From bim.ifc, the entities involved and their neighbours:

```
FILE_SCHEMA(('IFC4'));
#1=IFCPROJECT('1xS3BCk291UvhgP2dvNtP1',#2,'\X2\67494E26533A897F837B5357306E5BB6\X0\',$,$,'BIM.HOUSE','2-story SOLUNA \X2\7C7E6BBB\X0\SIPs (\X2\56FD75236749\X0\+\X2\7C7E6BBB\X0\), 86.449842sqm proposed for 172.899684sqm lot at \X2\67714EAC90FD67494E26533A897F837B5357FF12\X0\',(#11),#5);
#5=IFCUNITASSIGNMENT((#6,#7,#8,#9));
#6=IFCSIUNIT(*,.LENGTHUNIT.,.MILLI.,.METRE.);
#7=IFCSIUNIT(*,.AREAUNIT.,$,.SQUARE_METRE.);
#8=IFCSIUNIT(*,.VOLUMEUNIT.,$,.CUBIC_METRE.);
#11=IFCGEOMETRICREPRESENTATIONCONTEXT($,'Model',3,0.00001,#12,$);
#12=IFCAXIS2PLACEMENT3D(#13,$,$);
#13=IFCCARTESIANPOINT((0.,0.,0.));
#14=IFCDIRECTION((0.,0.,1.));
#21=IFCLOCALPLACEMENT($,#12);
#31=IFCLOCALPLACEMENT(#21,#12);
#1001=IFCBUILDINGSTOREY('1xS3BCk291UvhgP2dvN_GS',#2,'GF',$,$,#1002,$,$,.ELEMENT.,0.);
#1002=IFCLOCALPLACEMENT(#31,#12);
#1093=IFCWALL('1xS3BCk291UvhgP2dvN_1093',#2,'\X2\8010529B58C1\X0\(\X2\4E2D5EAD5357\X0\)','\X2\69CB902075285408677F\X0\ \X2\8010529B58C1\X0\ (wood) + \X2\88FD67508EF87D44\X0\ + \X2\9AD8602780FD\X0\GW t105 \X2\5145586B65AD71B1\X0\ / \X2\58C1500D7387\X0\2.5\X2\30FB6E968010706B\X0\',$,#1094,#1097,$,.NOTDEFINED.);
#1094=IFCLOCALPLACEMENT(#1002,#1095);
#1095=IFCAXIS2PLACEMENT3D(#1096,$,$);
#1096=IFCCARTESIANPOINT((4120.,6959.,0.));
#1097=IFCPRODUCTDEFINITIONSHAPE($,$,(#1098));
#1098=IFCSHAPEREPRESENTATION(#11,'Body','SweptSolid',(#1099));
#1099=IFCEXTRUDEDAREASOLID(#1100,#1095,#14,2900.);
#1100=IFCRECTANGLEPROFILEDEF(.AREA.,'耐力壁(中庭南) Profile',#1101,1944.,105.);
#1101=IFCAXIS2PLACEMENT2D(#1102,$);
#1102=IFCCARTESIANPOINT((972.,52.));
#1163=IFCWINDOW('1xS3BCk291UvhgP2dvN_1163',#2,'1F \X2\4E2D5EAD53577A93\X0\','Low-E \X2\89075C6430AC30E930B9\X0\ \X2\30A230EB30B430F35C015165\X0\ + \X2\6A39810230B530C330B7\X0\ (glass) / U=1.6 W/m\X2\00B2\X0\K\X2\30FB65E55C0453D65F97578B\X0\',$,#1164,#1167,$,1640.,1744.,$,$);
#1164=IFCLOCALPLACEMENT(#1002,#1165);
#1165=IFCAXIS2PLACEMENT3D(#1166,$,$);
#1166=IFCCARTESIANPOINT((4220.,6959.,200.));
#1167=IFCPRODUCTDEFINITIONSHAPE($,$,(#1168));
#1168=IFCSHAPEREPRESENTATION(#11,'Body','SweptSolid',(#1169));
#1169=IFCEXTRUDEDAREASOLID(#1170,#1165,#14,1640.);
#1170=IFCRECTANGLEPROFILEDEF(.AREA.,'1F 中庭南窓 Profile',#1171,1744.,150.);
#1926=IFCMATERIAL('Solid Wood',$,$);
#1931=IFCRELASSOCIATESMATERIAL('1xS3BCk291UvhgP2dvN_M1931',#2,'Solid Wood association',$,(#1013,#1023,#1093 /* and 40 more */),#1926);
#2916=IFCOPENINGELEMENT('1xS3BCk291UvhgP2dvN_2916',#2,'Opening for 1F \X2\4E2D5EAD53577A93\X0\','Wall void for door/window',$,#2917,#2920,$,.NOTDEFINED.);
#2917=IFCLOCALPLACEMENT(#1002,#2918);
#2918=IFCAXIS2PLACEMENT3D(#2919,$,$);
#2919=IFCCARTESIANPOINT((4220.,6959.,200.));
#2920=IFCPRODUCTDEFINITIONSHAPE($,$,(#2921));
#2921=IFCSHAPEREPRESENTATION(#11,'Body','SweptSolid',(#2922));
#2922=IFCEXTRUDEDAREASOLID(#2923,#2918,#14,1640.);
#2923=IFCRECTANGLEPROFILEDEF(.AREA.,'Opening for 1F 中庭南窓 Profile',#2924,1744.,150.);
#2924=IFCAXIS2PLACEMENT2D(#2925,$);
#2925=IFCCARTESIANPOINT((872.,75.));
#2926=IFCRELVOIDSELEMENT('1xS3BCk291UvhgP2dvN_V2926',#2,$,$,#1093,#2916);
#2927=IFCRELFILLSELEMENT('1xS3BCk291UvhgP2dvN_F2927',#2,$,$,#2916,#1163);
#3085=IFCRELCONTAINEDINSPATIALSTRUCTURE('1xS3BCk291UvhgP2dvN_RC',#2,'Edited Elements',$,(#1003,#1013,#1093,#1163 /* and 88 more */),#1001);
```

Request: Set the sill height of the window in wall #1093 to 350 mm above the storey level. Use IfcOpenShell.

```python
import numpy as np
import ifcopenshell
import ifcopenshell.api.geometry
import ifcopenshell.geom
import ifcopenshell.util.element
import ifcopenshell.util.placement
import ifcopenshell.util.shape
import ifcopenshell.util.unit

model = ifcopenshell.open("bim.ifc")
unit_scale = ifcopenshell.util.unit.calculate_unit_scale(model)

window = model.by_guid("1xS3BCk291UvhgP2dvN_1163")
opening = window.FillsVoids[0].RelatingOpeningElement
storey = ifcopenshell.util.element.get_container(window, ifc_class="IfcBuildingStorey")
level = ifcopenshell.util.placement.get_local_placement(storey.ObjectPlacement)[2, 3]

# The opening's origin need not be at the sill, so measure its lowest point.
shape = ifcopenshell.geom.create_shape(ifcopenshell.geom.settings(), opening)
bottom = ifcopenshell.util.shape.get_shape_bottom_elevation(shape, shape.geometry) / unit_scale
dz = level + 350.0 - bottom

shift = np.array([0.0, 0.0, dz])
# The window is not placed relative to its opening, so move both.
for product in (opening, window):
    matrix = ifcopenshell.util.placement.get_local_placement(product.ObjectPlacement)
    matrix[:3, 3] += shift
    ifcopenshell.api.geometry.edit_object_placement(model, product=product, matrix=matrix, is_si=False)

print(f"moved by {dz * unit_scale:+.3f} m")

model.write("bim-out.ifc")
```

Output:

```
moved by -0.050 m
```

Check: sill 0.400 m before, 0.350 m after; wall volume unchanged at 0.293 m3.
